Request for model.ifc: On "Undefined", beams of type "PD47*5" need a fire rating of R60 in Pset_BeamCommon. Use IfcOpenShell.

First a look at what the model holds.

```python
import ifcopenshell
import ifcopenshell.util.element

model = ifcopenshell.open("model.ifc")
print(model.schema)
storey = next(s for s in model.by_type("IfcBuildingStorey") if s.Name == "Undefined")
beams = [e for e in ifcopenshell.util.element.get_decomposition(storey) if e.is_a("IfcBeam")]
seen = {}
for e in beams:
    element_type = ifcopenshell.util.element.get_type(e)
    key = (element_type.Name if element_type != e and element_type else None, ifcopenshell.util.element.get_pset(e, "Pset_BeamCommon", "FireRating"))
    seen[key] = seen.get(key, 0) + 1
for (name, value), count in sorted(seen.items(), key=str):
    print(count, "x", name, "|", value)
```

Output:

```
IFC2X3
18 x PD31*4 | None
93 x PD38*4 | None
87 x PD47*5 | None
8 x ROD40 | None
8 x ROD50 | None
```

```python
import ifcopenshell
import ifcopenshell.api.pset
import ifcopenshell.util.element

model = ifcopenshell.open("model.ifc")

storey = next(s for s in model.by_type("IfcBuildingStorey") if s.Name == "Undefined")
beams = [e for e in ifcopenshell.util.element.get_decomposition(storey) if e.is_a("IfcBeam")]

count = 0
for e in beams:
    element_type = ifcopenshell.util.element.get_type(e)
    if element_type in (None, e) or element_type.Name != "PD47*5":
        continue
    found = ifcopenshell.util.element.get_pset(e, "Pset_BeamCommon", should_inherit=False)
    if found:
        pset = model.by_id(found["id"])
        if len(ifcopenshell.util.element.get_elements_by_pset(pset)) > 1:
            pset = ifcopenshell.api.pset.unshare_pset(model, products=[e], pset=pset)[0]
    else:
        pset = ifcopenshell.api.pset.add_pset(model, product=e, name="Pset_BeamCommon")
    ifcopenshell.api.pset.edit_pset(model, pset=pset, properties={"FireRating": "R60"})
    count += 1

print(count, "beams updated")

model.write("model-out.ifc")
```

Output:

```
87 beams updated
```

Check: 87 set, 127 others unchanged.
